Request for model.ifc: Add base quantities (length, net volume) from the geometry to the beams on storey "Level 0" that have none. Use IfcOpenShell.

First a look at what the model holds.

```python
import ifcopenshell
import ifcopenshell.util.element
import ifcopenshell.util.unit

model = ifcopenshell.open("model.ifc")
print(model.schema)
for unit_type in ("LENGTHUNIT", "AREAUNIT", "VOLUMEUNIT"):
    print(unit_type, ifcopenshell.util.unit.calculate_unit_scale(model, unit_type))
storey = next(s for s in model.by_type("IfcBuildingStorey") if s.Name == "Level 0")
beams = [e for e in ifcopenshell.util.element.get_decomposition(storey) if e.is_a("IfcBeam")]
for e in sorted(beams, key=lambda e: e.id()):
    print(e.id(), e.is_a(), e.Name, list(ifcopenshell.util.element.get_psets(e, qtos_only=True)), sep=" | ")
```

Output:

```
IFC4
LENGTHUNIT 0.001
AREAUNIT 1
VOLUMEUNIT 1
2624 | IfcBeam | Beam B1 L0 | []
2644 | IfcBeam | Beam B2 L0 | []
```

```python
import ifcopenshell
import ifcopenshell.api.pset
import ifcopenshell.geom
import ifcopenshell.util.element
import ifcopenshell.util.shape
import ifcopenshell.util.unit

model = ifcopenshell.open("model.ifc")
unit_scale = ifcopenshell.util.unit.calculate_unit_scale(model)
volume_scale = ifcopenshell.util.unit.calculate_unit_scale(model, "VOLUMEUNIT")
settings = ifcopenshell.geom.settings()

storey = next(s for s in model.by_type("IfcBuildingStorey") if s.Name == "Level 0")
beams = [e for e in ifcopenshell.util.element.get_decomposition(storey) if e.is_a("IfcBeam")]

for e in sorted(beams, key=lambda e: e.id()):
    if ifcopenshell.util.element.get_psets(e, qtos_only=True, should_inherit=False):
        continue
    # Geometry comes back in metres, in the element's own axes.
    shape = ifcopenshell.geom.create_shape(settings, e)
    values = {
        "Length": ifcopenshell.util.shape.get_max_xyz(shape.geometry) / unit_scale,
        "NetVolume": ifcopenshell.util.shape.get_volume(shape.geometry) / volume_scale,
    }
    qto = ifcopenshell.api.pset.add_qto(model, product=e, name="Qto_BeamBaseQuantities")
    ifcopenshell.api.pset.edit_qto(model, qto=qto, properties=values)
    print(e.id(), {k: round(v, 3) for k, v in values.items()})

model.write("model_rev.ifc")
```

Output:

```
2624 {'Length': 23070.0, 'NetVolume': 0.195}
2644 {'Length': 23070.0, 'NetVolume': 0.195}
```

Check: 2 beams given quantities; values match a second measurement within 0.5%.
